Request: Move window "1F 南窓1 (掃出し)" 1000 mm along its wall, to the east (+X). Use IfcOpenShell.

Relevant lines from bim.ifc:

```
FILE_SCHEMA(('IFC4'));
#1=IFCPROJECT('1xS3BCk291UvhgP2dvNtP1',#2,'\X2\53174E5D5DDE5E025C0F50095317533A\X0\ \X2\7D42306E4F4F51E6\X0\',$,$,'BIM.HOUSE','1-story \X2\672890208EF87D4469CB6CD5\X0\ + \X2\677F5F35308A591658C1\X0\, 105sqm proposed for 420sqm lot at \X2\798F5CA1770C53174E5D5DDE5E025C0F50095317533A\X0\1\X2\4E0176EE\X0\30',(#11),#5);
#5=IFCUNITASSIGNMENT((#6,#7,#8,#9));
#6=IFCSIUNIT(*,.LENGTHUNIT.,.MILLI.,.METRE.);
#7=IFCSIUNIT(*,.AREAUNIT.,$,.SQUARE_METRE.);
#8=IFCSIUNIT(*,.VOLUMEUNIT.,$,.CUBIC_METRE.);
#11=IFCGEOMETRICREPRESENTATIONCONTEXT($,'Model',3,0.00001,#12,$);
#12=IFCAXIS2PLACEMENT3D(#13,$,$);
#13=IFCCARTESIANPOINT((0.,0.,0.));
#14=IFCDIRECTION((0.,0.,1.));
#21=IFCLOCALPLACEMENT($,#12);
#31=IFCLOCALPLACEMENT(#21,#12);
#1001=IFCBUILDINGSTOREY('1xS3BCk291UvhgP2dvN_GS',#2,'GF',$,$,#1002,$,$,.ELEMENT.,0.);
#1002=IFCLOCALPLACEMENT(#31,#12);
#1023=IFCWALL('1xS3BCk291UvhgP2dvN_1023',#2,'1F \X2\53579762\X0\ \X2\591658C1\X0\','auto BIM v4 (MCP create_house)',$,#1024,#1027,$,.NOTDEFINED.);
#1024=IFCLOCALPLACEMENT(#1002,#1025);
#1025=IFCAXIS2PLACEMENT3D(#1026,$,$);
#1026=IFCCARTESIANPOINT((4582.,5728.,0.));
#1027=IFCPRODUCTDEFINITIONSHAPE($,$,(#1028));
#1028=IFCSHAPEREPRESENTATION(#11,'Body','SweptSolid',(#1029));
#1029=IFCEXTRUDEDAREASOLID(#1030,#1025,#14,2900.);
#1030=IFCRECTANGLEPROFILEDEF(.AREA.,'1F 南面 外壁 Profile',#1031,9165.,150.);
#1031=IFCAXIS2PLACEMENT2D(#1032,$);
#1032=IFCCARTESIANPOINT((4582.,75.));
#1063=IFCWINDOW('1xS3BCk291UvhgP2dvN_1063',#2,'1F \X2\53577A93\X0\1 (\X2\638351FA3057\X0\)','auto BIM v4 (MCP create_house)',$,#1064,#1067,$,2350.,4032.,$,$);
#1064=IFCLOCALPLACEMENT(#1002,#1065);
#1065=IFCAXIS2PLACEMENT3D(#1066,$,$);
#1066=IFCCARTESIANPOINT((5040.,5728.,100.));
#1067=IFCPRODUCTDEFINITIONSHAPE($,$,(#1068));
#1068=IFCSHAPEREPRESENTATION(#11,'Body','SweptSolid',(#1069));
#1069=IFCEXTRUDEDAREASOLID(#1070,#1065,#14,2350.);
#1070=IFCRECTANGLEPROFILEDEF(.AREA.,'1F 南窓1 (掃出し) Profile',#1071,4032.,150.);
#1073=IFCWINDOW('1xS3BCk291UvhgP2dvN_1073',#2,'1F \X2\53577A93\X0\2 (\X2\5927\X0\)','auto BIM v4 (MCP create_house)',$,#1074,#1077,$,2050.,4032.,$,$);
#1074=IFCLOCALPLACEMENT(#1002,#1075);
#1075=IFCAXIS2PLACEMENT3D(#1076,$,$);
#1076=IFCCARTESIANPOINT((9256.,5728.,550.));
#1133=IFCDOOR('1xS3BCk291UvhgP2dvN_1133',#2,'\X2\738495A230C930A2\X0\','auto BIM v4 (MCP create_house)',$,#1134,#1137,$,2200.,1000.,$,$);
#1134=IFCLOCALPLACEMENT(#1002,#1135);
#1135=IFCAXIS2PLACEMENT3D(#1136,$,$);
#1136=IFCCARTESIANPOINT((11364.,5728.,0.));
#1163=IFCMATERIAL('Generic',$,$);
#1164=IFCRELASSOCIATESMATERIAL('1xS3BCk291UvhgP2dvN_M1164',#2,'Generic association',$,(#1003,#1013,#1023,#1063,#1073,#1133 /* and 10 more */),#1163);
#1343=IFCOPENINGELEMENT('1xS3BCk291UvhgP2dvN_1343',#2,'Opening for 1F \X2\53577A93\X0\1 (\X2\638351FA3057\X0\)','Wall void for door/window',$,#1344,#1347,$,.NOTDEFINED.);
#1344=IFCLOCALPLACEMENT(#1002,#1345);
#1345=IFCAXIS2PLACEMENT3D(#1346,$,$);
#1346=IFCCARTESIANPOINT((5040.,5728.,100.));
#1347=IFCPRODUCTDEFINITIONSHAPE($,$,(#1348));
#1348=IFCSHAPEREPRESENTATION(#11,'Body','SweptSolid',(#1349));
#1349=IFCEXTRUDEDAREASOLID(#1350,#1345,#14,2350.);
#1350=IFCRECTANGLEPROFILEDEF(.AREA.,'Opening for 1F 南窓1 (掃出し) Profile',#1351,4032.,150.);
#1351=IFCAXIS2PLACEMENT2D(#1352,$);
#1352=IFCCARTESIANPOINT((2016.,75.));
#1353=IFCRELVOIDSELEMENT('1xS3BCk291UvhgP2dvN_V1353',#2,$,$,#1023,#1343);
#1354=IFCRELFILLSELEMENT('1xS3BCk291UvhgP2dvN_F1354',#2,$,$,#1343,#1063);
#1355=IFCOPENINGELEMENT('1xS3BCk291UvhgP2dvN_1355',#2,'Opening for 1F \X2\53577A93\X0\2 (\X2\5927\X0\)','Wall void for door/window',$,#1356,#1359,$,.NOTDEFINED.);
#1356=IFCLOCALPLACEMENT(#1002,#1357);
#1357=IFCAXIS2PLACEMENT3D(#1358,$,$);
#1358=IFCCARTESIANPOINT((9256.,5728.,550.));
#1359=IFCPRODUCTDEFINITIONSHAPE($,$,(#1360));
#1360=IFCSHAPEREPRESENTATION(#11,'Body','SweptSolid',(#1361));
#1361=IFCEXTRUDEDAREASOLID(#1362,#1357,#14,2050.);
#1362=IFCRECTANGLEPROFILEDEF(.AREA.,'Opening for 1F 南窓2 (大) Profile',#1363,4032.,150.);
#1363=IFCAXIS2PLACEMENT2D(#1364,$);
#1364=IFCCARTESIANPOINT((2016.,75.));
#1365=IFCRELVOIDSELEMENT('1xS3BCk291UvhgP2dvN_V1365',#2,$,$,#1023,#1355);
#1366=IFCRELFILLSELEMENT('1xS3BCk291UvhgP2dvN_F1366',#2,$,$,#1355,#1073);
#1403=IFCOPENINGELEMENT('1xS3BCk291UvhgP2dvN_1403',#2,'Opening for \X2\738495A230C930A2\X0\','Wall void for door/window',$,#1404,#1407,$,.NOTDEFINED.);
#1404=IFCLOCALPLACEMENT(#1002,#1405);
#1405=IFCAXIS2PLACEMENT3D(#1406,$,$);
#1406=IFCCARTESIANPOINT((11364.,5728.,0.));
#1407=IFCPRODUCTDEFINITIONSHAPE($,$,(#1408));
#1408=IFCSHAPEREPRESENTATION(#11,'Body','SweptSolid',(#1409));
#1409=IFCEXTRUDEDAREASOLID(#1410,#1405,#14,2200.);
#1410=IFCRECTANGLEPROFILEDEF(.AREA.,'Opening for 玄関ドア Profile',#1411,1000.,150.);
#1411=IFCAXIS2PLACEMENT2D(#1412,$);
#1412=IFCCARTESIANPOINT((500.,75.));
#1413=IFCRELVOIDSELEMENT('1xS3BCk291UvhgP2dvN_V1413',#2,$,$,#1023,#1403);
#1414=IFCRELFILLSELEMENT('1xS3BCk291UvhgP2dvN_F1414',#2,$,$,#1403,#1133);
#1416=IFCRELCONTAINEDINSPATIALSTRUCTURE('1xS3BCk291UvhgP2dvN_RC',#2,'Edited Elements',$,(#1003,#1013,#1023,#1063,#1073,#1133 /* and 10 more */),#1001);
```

```python
import ifcopenshell
import ifcopenshell.api.geometry
import ifcopenshell.util.placement
import ifcopenshell.util.unit

model = ifcopenshell.open("bim.ifc")
unit_scale = ifcopenshell.util.unit.calculate_unit_scale(model)

window = model.by_guid("1xS3BCk291UvhgP2dvN_1063")
opening = window.FillsVoids[0].RelatingOpeningElement
wall = opening.VoidsElements[0].RelatingBuildingElement

wall_matrix = ifcopenshell.util.placement.get_local_placement(wall.ObjectPlacement)
shift = wall_matrix[:3, 0] * 1 / unit_scale
before = ifcopenshell.util.placement.get_local_placement(window.ObjectPlacement)[:3, 3].copy()

# The window is not placed relative to its opening, so move both.
for product in (opening, window):
    matrix = ifcopenshell.util.placement.get_local_placement(product.ObjectPlacement)
    matrix[:3, 3] += shift
    ifcopenshell.api.geometry.edit_object_placement(model, product=product, matrix=matrix, is_si=False)

after = ifcopenshell.util.placement.get_local_placement(window.ObjectPlacement)[:3, 3]
print("window moved by", (after - before).round(3) + 0.0)

model.write("bim-out.ifc")
```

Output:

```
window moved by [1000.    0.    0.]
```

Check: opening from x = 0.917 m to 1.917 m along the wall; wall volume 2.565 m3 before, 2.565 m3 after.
